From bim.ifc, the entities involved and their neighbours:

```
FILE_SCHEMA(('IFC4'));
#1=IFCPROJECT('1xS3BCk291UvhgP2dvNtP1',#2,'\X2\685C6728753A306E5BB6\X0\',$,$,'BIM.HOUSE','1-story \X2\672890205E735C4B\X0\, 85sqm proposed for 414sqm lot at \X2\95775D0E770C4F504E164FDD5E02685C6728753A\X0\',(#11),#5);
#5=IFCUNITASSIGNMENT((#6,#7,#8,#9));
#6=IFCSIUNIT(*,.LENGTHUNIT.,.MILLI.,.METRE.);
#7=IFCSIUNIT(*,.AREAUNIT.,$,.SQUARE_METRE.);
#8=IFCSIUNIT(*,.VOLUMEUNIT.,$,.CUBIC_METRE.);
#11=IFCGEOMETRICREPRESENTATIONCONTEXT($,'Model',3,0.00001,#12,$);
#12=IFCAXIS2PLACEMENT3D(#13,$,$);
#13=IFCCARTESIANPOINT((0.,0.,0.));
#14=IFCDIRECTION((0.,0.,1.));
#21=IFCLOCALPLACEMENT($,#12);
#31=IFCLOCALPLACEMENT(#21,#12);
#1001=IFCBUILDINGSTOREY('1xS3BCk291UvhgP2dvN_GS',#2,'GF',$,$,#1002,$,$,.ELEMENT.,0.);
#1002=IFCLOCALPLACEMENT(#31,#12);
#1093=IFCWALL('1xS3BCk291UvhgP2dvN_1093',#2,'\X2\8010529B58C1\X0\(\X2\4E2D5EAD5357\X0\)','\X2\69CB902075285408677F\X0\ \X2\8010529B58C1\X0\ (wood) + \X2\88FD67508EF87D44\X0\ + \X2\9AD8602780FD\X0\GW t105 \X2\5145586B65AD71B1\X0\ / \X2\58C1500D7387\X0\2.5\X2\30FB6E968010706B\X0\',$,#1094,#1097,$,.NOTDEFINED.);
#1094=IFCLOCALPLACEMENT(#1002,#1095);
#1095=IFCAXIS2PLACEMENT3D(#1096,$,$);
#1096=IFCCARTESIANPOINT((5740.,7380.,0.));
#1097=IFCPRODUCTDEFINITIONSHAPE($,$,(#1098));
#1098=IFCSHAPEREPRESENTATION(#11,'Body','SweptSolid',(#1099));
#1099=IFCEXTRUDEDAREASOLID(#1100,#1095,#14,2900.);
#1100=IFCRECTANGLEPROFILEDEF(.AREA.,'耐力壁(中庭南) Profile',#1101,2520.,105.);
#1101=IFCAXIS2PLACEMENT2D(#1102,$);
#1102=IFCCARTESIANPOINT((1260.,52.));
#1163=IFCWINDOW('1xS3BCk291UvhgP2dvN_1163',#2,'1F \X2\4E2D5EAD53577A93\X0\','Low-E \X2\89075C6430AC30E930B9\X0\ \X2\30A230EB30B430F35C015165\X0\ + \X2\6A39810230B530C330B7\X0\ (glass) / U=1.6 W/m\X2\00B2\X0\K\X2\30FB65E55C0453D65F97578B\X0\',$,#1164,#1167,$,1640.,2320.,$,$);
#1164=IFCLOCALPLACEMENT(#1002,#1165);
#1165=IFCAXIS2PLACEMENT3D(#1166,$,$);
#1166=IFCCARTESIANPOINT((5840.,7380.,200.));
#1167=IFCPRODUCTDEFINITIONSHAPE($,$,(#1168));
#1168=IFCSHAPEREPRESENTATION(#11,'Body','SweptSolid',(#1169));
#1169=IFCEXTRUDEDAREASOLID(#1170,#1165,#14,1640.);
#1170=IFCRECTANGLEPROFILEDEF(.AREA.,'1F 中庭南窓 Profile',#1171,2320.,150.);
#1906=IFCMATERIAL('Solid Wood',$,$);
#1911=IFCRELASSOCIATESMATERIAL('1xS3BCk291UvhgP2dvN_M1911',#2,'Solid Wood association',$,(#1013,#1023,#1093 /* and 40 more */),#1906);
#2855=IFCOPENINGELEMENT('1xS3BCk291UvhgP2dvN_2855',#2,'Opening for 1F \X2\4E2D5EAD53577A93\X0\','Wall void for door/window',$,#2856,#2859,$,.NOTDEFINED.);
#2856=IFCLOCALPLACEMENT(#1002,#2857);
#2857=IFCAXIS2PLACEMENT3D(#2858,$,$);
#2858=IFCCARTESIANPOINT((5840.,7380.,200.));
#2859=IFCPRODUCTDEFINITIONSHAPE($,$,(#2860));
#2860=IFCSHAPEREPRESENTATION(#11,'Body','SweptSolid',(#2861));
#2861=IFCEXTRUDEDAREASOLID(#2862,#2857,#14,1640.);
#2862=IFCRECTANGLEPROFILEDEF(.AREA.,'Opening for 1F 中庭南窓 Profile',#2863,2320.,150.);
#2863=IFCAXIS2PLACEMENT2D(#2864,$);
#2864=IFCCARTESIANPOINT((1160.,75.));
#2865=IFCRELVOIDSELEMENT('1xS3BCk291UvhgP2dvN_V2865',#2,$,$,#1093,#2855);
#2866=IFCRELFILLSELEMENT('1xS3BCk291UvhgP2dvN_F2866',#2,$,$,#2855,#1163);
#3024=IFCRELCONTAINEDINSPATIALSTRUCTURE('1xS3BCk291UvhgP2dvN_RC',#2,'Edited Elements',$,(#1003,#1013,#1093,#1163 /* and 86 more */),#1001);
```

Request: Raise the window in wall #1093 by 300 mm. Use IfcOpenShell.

```python
import numpy as np
import ifcopenshell
import ifcopenshell.api.geometry
import ifcopenshell.util.placement
import ifcopenshell.util.unit

model = ifcopenshell.open("bim.ifc")
unit_scale = ifcopenshell.util.unit.calculate_unit_scale(model)

window = model.by_guid("1xS3BCk291UvhgP2dvN_1163")
opening = window.FillsVoids[0].RelatingOpeningElement
dz = 300.0

shift = np.array([0.0, 0.0, dz])
# The window is not placed relative to its opening, so move both.
for product in (opening, window):
    matrix = ifcopenshell.util.placement.get_local_placement(product.ObjectPlacement)
    matrix[:3, 3] += shift
    ifcopenshell.api.geometry.edit_object_placement(model, product=product, matrix=matrix, is_si=False)

print(f"moved by {dz * unit_scale:+.3f} m")

model.write("bim_rev.ifc")
```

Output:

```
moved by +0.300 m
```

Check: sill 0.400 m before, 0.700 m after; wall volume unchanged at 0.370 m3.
